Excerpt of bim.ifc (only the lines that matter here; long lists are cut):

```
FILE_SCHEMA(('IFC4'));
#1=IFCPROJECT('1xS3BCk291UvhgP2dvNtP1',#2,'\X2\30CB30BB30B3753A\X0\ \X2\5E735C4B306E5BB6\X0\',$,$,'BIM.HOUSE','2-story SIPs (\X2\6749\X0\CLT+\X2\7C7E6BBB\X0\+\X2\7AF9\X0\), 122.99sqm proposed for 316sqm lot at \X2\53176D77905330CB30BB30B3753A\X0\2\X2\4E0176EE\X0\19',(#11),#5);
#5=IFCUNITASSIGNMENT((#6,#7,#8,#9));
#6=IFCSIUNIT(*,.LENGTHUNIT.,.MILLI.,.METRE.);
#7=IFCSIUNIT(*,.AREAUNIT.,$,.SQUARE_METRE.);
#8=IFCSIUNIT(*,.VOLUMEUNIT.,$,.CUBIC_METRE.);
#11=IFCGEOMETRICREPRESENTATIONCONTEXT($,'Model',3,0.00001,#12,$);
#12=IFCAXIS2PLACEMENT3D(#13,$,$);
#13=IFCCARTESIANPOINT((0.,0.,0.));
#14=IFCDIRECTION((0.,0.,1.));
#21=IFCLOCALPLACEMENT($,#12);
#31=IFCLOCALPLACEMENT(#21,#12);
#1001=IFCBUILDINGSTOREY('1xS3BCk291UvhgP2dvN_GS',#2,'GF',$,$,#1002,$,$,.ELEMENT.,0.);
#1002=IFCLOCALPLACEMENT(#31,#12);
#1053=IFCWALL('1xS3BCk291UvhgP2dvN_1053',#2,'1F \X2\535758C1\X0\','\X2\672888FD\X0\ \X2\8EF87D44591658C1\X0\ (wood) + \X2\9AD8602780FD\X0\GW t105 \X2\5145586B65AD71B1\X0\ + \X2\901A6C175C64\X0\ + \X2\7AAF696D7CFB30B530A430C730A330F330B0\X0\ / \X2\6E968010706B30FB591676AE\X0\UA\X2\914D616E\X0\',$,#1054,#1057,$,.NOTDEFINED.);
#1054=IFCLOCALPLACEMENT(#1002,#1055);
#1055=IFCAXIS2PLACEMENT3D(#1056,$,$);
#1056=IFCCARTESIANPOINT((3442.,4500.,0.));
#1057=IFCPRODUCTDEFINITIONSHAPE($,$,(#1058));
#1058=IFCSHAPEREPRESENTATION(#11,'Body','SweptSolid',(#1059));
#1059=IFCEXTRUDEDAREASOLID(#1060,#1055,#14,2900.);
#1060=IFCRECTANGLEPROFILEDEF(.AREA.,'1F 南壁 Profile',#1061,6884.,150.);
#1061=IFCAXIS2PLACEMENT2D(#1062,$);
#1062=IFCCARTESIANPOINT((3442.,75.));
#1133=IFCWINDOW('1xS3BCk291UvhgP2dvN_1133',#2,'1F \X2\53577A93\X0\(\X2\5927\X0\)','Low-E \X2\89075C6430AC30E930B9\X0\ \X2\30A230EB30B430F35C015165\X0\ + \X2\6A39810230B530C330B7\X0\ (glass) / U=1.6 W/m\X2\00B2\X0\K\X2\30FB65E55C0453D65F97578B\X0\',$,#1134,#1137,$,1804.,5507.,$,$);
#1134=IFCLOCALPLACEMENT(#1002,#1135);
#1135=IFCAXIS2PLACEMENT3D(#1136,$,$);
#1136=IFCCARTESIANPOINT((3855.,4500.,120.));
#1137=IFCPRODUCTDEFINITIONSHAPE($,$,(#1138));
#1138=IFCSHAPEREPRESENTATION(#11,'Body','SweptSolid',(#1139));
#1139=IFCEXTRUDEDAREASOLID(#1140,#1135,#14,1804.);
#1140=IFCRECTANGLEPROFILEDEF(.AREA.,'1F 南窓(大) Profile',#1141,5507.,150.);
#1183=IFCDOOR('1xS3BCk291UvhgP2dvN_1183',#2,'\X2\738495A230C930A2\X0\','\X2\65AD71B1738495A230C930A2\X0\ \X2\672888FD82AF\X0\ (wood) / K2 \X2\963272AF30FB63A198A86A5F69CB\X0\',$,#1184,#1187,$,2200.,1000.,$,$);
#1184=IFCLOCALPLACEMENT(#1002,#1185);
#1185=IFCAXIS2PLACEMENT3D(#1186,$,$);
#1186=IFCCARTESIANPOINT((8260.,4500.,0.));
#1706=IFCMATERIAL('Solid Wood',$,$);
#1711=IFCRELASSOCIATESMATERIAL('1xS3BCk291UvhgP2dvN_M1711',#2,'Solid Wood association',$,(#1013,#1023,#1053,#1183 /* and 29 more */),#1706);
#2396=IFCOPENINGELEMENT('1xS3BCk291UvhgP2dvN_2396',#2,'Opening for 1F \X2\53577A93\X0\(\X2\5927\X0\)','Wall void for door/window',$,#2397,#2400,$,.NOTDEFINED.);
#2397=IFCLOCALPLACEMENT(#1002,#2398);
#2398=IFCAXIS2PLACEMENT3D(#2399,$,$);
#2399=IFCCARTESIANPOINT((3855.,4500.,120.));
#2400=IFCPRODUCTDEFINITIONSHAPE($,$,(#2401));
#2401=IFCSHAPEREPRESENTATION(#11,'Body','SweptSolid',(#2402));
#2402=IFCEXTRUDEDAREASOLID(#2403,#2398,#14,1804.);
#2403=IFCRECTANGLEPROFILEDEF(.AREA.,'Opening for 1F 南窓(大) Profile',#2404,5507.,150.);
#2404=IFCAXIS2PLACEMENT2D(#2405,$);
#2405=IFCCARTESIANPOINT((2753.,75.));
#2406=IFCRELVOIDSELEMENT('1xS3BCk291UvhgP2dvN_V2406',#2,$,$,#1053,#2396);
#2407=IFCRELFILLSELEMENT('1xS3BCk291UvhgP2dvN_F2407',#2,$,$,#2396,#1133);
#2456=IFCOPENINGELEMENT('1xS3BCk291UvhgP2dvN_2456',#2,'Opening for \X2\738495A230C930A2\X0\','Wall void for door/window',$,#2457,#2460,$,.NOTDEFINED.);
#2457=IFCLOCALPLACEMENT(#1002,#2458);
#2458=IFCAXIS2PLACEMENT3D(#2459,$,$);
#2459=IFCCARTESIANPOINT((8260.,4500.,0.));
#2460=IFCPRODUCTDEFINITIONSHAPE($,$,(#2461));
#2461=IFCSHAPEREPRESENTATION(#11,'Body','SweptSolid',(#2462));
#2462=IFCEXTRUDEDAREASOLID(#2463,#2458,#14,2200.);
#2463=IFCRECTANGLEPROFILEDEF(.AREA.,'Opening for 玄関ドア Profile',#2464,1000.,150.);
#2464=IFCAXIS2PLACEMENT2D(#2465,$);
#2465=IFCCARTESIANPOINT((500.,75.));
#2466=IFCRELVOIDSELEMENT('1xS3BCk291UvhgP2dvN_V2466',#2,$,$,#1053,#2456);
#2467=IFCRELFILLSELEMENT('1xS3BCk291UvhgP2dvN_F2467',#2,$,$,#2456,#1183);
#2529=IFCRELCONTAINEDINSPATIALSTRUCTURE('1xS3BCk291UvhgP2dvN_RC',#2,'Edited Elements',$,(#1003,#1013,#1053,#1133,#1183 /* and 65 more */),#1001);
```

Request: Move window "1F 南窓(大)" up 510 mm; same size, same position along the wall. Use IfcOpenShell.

```python
import numpy as np
import ifcopenshell
import ifcopenshell.api.geometry
import ifcopenshell.util.placement
import ifcopenshell.util.unit

model = ifcopenshell.open("bim.ifc")
unit_scale = ifcopenshell.util.unit.calculate_unit_scale(model)

window = model.by_guid("1xS3BCk291UvhgP2dvN_1133")
opening = window.FillsVoids[0].RelatingOpeningElement
dz = 0.51 / unit_scale

shift = np.array([0.0, 0.0, dz])
# The window is not placed relative to its opening, so move both.
for product in (opening, window):
    matrix = ifcopenshell.util.placement.get_local_placement(product.ObjectPlacement)
    matrix[:3, 3] += shift
    ifcopenshell.api.geometry.edit_object_placement(model, product=product, matrix=matrix, is_si=False)

print(f"moved by {dz * unit_scale:+.3f} m")

model.write("bim-out.ifc")
```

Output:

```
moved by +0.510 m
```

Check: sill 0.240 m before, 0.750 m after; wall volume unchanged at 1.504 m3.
